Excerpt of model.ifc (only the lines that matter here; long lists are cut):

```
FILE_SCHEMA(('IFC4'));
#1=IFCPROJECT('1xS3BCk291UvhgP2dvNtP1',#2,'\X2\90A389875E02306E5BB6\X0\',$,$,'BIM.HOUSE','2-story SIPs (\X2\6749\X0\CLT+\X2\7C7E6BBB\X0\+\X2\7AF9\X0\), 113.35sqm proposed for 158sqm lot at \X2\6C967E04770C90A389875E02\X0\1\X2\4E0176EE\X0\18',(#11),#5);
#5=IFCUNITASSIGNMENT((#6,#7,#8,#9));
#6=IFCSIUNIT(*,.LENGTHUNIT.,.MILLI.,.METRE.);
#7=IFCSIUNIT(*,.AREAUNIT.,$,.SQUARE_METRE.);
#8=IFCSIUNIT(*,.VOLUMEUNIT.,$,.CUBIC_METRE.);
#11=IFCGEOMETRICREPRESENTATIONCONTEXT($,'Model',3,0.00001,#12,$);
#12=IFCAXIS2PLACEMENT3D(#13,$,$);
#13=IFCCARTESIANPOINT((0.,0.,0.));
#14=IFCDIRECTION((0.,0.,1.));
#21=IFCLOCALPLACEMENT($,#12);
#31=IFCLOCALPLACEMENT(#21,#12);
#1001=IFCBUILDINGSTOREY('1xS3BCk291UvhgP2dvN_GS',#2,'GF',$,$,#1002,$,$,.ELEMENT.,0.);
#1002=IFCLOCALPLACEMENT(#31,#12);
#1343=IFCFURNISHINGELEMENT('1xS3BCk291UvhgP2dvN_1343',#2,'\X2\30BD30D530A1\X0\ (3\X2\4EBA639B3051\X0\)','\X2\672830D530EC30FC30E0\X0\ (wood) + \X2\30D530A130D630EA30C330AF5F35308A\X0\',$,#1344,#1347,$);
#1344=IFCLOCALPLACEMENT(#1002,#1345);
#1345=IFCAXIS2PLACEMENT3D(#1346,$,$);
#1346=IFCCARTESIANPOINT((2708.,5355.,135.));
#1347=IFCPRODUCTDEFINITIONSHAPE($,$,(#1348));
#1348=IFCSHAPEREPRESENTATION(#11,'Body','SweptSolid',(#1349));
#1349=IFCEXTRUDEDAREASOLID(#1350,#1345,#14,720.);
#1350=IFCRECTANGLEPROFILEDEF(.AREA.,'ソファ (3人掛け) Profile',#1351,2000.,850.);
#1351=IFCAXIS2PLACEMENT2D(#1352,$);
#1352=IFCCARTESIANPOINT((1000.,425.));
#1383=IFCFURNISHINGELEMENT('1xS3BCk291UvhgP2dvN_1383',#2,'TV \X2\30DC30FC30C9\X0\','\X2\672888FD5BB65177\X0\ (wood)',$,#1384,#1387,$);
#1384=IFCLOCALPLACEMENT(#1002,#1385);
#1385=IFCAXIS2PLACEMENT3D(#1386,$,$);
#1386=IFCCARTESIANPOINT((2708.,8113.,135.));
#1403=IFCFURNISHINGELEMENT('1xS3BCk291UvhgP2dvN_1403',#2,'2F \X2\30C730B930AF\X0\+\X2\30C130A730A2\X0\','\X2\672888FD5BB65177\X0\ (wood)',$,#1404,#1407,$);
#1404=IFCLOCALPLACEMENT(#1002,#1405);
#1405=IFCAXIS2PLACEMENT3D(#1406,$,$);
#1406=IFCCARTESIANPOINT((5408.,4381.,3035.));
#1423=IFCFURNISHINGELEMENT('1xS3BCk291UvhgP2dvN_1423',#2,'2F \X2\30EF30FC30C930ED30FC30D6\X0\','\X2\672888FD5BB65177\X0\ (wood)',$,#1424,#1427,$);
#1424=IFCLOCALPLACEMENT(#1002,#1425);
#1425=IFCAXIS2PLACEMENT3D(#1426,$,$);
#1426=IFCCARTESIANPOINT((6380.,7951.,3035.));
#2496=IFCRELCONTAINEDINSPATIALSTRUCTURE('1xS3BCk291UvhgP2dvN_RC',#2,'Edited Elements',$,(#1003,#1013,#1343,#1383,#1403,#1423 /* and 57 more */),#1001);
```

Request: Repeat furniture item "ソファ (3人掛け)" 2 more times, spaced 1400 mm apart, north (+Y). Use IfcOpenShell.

```python
import numpy as np
import ifcopenshell
import ifcopenshell.api.geometry
import ifcopenshell.api.root
import ifcopenshell.util.element
import ifcopenshell.util.placement

model = ifcopenshell.open("model.ifc")


def reuse_history(source, copy):
    """copy_class also copies each property set's owner history, people and application; keep the originals."""
    for rel in copy.IsDefinedBy:
        if rel.is_a("IfcRelDefinesByProperties") and (history := rel.RelatingPropertyDefinition.OwnerHistory):
            rel.RelatingPropertyDefinition.OwnerHistory = source.OwnerHistory
            ifcopenshell.util.element.remove_deep2(model, history)


source = model.by_id(1343)
base = ifcopenshell.util.placement.get_local_placement(source.ObjectPlacement)
step = np.array([0.0, 1.0, 0.0]) * 1400.0

for i in range(1, 3):
    copy = ifcopenshell.api.root.copy_class(model, product=source)
    copy.Representation = ifcopenshell.util.element.copy_deep(
        model, source.Representation, exclude=["IfcGeometricRepresentationContext", "IfcRepresentationMap"]
    )
    reuse_history(source, copy)
    matrix = base.copy()
    matrix[:3, 3] += i * step
    print("added at", matrix[:3, 3].round(3) + 0.0)
    ifcopenshell.api.geometry.edit_object_placement(model, product=copy, matrix=matrix, is_si=False)

model.write("model_updated.ifc")
```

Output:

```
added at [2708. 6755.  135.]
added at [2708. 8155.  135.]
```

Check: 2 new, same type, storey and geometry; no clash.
